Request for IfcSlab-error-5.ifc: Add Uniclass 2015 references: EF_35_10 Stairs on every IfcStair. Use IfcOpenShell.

First a look at what the model holds.

```python
import ifcopenshell

model = ifcopenshell.open("IfcSlab-error-5.ifc")
print(model.schema)
print("classifications:", [c.Name for c in model.by_type("IfcClassification")])
for ifc_class in ("IfcDoor", "IfcRoof", "IfcStair", "IfcWall", "IfcWindow"):
    print(ifc_class, len(model.by_type(ifc_class)))
```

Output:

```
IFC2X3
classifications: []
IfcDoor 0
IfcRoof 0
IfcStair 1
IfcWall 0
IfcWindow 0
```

```python
import ifcopenshell
import ifcopenshell.api.classification

model = ifcopenshell.open("IfcSlab-error-5.ifc")

# IFC2X3 requires Source and Edition and has no link from the project to the system.
system = model.create_entity("IfcClassification", Source="NBS", Edition="2015", Name="Uniclass 2015")

codes = {
    "IfcStair": ("EF_35_10", "Stairs"),
}
for ifc_class, (code, name) in codes.items():
    products = model.by_type(ifc_class)
    ifcopenshell.api.classification.add_reference(
        model, products=products, classification=system, identification=code, name=name
    )
    print(code, len(products))

model.write("IfcSlab-error-5_updated.ifc")
```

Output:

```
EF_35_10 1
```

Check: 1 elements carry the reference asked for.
